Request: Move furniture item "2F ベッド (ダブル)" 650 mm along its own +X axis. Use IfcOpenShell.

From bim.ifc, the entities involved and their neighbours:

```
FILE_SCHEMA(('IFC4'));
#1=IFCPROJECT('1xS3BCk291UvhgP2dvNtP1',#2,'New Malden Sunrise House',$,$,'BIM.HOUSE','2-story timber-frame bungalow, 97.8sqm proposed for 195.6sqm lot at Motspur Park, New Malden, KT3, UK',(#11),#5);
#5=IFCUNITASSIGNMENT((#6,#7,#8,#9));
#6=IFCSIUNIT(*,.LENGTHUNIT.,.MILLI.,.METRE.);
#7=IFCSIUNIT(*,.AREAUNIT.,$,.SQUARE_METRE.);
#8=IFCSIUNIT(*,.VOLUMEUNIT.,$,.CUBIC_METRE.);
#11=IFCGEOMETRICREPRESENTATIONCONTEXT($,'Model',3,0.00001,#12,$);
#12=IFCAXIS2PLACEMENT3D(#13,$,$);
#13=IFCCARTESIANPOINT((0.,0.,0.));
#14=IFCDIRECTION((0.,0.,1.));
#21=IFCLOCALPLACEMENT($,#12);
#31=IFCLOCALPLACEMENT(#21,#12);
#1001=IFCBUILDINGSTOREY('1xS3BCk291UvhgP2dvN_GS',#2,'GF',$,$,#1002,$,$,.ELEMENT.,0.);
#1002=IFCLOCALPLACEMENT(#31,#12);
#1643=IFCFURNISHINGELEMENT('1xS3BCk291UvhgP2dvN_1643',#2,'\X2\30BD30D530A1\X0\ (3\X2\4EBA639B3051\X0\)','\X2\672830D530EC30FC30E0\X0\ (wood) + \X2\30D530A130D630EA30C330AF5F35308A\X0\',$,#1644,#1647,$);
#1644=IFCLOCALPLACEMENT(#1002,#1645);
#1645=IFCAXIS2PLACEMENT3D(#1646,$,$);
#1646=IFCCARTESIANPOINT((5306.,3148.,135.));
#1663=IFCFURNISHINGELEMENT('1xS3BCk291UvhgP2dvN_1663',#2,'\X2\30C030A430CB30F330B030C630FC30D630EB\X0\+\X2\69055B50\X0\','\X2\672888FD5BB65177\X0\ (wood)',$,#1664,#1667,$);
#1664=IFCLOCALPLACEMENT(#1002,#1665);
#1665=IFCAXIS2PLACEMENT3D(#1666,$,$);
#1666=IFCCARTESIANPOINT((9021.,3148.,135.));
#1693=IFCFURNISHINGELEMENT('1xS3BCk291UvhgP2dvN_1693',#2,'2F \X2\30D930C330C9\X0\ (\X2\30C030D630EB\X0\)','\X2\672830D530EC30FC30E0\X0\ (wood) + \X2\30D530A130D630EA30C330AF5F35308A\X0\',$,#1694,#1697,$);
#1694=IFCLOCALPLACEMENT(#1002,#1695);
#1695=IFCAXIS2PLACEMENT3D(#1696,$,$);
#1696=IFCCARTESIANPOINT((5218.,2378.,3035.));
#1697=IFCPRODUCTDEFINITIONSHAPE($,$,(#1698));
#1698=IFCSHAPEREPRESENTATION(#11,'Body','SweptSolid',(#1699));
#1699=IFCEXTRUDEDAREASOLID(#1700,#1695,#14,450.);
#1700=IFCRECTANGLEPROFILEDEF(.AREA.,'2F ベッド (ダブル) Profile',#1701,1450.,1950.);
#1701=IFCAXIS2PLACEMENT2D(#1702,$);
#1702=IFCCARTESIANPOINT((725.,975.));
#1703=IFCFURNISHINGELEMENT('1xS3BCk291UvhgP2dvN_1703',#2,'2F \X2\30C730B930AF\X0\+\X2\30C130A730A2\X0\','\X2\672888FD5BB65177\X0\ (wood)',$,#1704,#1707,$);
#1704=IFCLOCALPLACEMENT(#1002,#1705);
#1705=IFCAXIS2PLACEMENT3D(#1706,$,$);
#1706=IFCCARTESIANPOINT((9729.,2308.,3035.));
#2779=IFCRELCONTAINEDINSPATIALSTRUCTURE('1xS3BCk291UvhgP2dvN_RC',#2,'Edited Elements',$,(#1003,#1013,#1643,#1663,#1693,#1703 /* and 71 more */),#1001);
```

```python
import ifcopenshell
import ifcopenshell.api.geometry
import ifcopenshell.util.placement
import ifcopenshell.util.unit

model = ifcopenshell.open("bim.ifc")
unit_scale = ifcopenshell.util.unit.calculate_unit_scale(model)

item = model.by_id(1693)
matrix = ifcopenshell.util.placement.get_local_placement(item.ObjectPlacement)
matrix[:3, 3] += matrix[:3, 0] * 0.65 / unit_scale
ifcopenshell.api.geometry.edit_object_placement(model, product=item, matrix=matrix, is_si=False)

print(ifcopenshell.util.placement.get_local_placement(item.ObjectPlacement).round(3) + 0.0)

model.write("bim_rev.ifc")
```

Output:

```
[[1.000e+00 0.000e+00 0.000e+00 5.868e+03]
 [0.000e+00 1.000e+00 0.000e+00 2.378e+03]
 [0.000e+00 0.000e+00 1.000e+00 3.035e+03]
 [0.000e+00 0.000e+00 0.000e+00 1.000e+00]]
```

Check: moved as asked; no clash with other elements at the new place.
